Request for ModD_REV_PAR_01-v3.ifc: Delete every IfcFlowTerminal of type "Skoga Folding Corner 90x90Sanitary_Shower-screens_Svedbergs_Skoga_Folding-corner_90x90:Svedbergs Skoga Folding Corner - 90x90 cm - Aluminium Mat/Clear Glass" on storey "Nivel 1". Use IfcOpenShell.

First a look at what the model holds.

```python
import ifcopenshell
import ifcopenshell.util.element

model = ifcopenshell.open("ModD_REV_PAR_01-v3.ifc")
print(model.schema)
storey = next(s for s in model.by_type("IfcBuildingStorey") if s.Name == "Nivel 1")
terminals = [e for e in ifcopenshell.util.element.get_decomposition(storey) if e.is_a("IfcFlowTerminal")]
seen = {}
for e in terminals:
    element_type = ifcopenshell.util.element.get_type(e)
    name = element_type.Name if element_type not in (None, e) else None
    seen[name] = seen.get(name, 0) + 1
for name, count in sorted(seen.items(), key=str):
    print(count, "x", name)
```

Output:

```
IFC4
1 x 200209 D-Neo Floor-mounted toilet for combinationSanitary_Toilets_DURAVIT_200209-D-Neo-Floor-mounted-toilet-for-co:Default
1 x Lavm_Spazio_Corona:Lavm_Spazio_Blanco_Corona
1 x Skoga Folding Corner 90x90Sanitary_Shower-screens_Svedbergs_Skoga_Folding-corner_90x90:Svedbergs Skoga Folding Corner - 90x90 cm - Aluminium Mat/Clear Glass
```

```python
import ifcopenshell
import ifcopenshell.api.root
import ifcopenshell.util.element

model = ifcopenshell.open("ModD_REV_PAR_01-v3.ifc")

storey = next(s for s in model.by_type("IfcBuildingStorey") if s.Name == "Nivel 1")
terminals = [e for e in ifcopenshell.util.element.get_decomposition(storey) if e.is_a("IfcFlowTerminal")]
targets = [e for e in terminals if (t := ifcopenshell.util.element.get_type(e)) not in (None, e) and t.Name == "Skoga Folding Corner 90x90Sanitary_Shower-screens_Svedbergs_Skoga_Folding-corner_90x90:Svedbergs Skoga Folding Corner - 90x90 cm - Aluminium Mat/Clear Glass"]

for e in targets:
    ifcopenshell.api.root.remove_product(model, product=e)
print(len(targets), "removed")

model.write("ModD_REV_PAR_01-v3-out.ifc")
```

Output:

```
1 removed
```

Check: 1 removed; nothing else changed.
